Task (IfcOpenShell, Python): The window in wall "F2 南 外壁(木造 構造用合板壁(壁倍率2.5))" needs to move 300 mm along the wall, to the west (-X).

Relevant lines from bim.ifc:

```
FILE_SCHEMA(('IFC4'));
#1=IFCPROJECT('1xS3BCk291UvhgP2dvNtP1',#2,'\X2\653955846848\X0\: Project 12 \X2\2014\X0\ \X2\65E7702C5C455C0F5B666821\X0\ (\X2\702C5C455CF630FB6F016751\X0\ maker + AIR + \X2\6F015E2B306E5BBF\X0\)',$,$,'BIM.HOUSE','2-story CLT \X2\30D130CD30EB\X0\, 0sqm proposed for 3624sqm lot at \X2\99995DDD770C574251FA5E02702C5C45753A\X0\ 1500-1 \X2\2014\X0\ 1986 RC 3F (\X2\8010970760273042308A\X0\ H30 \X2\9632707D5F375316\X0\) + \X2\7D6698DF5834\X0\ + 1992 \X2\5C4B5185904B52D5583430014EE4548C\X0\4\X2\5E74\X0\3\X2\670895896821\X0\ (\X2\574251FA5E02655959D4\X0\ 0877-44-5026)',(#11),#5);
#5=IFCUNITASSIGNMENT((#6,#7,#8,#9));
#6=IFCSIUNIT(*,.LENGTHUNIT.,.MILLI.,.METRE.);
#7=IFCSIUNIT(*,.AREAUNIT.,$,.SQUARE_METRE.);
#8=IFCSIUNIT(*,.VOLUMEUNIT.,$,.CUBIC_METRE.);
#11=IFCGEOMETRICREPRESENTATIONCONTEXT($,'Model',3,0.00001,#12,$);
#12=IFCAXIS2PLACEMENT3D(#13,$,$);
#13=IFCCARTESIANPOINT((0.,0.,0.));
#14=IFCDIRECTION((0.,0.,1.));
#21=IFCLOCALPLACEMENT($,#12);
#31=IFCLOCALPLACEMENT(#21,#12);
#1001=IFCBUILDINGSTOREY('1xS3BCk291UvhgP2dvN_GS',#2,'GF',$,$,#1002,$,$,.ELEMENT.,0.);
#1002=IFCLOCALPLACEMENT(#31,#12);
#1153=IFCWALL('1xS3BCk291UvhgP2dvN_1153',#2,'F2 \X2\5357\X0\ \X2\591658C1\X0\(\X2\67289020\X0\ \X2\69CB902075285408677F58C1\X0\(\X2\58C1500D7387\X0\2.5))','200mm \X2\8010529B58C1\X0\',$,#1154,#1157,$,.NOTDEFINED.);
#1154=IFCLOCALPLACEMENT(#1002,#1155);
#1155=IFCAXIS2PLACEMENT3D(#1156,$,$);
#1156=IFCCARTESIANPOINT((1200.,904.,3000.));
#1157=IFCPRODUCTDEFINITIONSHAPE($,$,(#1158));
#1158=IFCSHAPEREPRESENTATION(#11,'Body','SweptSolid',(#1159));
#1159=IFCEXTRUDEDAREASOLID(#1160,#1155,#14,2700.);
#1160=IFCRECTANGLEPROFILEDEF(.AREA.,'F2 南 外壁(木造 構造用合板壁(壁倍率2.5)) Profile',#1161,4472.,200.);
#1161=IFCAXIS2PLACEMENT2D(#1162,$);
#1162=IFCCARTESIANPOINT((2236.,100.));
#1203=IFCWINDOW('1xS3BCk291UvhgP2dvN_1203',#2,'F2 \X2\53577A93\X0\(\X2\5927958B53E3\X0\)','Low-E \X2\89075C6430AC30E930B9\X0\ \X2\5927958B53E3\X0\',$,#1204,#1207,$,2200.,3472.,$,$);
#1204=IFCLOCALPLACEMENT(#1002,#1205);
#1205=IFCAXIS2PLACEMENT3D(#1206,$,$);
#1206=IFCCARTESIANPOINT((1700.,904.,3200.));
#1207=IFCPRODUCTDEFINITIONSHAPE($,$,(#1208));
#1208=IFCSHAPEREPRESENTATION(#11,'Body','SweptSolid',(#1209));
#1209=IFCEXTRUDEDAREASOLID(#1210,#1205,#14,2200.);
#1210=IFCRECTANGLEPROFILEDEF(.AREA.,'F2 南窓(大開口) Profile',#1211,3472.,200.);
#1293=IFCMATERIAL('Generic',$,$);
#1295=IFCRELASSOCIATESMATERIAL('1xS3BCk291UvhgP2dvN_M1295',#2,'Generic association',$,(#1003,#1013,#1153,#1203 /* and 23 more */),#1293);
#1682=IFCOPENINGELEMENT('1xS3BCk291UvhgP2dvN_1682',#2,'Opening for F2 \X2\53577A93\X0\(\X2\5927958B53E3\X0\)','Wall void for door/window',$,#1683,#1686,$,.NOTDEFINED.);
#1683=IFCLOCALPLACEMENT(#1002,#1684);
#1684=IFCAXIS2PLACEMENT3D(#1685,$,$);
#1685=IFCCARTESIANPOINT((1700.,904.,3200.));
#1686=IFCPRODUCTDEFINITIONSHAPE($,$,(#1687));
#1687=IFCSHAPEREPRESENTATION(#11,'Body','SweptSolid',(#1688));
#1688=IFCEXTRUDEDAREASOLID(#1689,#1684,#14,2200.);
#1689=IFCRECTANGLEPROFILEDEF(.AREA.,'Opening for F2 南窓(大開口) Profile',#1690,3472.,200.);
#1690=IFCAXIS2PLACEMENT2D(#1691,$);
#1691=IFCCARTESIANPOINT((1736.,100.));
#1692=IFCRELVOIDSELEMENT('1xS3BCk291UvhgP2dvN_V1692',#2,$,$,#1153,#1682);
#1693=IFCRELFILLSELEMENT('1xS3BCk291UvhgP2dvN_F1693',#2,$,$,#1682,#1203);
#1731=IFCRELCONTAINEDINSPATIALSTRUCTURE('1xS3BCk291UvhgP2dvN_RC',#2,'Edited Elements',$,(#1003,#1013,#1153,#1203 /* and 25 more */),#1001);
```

```python
import ifcopenshell
import ifcopenshell.api.geometry
import ifcopenshell.util.placement
import ifcopenshell.util.unit

model = ifcopenshell.open("bim.ifc")
unit_scale = ifcopenshell.util.unit.calculate_unit_scale(model)

window = model.by_id(1203)
opening = window.FillsVoids[0].RelatingOpeningElement
wall = opening.VoidsElements[0].RelatingBuildingElement

wall_matrix = ifcopenshell.util.placement.get_local_placement(wall.ObjectPlacement)
shift = wall_matrix[:3, 0] * -0.3 / unit_scale
before = ifcopenshell.util.placement.get_local_placement(window.ObjectPlacement)[:3, 3].copy()

# The window is not placed relative to its opening, so move both.
for product in (opening, window):
    matrix = ifcopenshell.util.placement.get_local_placement(product.ObjectPlacement)
    matrix[:3, 3] += shift
    ifcopenshell.api.geometry.edit_object_placement(model, product=product, matrix=matrix, is_si=False)

after = ifcopenshell.util.placement.get_local_placement(window.ObjectPlacement)[:3, 3]
print("window moved by", (after - before).round(3) + 0.0)

model.write("bim_v2.ifc")
```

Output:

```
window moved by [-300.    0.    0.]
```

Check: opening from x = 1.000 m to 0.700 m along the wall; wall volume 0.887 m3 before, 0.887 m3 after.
